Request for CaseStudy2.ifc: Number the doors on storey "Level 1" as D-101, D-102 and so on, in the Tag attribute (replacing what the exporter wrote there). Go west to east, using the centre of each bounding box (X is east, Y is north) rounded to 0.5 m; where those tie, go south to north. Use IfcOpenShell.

First a look at what the model holds.

```python
import ifcopenshell
import ifcopenshell.util.element
import ifcopenshell.util.placement

model = ifcopenshell.open("CaseStudy2.ifc")
print(model.schema)
storey = next(s for s in model.by_type("IfcBuildingStorey") if s.Name == "Level 1")
doors = [e for e in ifcopenshell.util.element.get_decomposition(storey) if e.is_a("IfcDoor")]
for e in sorted(doors, key=lambda e: e.id()):
    origin = ifcopenshell.util.placement.get_local_placement(e.ObjectPlacement)[:3, 3]
    print(e.id(), e.Tag, e.Name, origin.round(2) + 0.0, sep=" | ")
```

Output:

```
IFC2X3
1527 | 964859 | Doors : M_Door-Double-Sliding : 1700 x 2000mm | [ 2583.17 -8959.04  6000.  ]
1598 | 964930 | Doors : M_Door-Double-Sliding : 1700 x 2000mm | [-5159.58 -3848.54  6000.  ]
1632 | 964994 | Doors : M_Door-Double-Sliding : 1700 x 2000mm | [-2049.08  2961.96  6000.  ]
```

```python
import ifcopenshell
import ifcopenshell.geom
import ifcopenshell.util.element
import ifcopenshell.util.shape

model = ifcopenshell.open("CaseStudy2.ifc")
settings = ifcopenshell.geom.settings()
settings.set("use-world-coords", True)


def centre(element):
    shape = ifcopenshell.geom.create_shape(settings, element)
    return ifcopenshell.util.shape.get_bbox_centroid(shape.geometry)


storey = next(s for s in model.by_type("IfcBuildingStorey") if s.Name == "Level 1")
doors = [e for e in ifcopenshell.util.element.get_decomposition(storey) if e.is_a("IfcDoor")]

# Insertion points can sit at a corner or the storey origin, so sort by the geometry (in metres).
centres = {e: centre(e) for e in doors}
doors.sort(key=lambda e: (round(centres[e][0] / 0.5), centres[e][1]))

for i, e in enumerate(doors, start=1):
    number = f"D-1{i:02d}"
    e.Tag = number
    print(e.id(), number)

model.write("CaseStudy2_v2.ifc")
```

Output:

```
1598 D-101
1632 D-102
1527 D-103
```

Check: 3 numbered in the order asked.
